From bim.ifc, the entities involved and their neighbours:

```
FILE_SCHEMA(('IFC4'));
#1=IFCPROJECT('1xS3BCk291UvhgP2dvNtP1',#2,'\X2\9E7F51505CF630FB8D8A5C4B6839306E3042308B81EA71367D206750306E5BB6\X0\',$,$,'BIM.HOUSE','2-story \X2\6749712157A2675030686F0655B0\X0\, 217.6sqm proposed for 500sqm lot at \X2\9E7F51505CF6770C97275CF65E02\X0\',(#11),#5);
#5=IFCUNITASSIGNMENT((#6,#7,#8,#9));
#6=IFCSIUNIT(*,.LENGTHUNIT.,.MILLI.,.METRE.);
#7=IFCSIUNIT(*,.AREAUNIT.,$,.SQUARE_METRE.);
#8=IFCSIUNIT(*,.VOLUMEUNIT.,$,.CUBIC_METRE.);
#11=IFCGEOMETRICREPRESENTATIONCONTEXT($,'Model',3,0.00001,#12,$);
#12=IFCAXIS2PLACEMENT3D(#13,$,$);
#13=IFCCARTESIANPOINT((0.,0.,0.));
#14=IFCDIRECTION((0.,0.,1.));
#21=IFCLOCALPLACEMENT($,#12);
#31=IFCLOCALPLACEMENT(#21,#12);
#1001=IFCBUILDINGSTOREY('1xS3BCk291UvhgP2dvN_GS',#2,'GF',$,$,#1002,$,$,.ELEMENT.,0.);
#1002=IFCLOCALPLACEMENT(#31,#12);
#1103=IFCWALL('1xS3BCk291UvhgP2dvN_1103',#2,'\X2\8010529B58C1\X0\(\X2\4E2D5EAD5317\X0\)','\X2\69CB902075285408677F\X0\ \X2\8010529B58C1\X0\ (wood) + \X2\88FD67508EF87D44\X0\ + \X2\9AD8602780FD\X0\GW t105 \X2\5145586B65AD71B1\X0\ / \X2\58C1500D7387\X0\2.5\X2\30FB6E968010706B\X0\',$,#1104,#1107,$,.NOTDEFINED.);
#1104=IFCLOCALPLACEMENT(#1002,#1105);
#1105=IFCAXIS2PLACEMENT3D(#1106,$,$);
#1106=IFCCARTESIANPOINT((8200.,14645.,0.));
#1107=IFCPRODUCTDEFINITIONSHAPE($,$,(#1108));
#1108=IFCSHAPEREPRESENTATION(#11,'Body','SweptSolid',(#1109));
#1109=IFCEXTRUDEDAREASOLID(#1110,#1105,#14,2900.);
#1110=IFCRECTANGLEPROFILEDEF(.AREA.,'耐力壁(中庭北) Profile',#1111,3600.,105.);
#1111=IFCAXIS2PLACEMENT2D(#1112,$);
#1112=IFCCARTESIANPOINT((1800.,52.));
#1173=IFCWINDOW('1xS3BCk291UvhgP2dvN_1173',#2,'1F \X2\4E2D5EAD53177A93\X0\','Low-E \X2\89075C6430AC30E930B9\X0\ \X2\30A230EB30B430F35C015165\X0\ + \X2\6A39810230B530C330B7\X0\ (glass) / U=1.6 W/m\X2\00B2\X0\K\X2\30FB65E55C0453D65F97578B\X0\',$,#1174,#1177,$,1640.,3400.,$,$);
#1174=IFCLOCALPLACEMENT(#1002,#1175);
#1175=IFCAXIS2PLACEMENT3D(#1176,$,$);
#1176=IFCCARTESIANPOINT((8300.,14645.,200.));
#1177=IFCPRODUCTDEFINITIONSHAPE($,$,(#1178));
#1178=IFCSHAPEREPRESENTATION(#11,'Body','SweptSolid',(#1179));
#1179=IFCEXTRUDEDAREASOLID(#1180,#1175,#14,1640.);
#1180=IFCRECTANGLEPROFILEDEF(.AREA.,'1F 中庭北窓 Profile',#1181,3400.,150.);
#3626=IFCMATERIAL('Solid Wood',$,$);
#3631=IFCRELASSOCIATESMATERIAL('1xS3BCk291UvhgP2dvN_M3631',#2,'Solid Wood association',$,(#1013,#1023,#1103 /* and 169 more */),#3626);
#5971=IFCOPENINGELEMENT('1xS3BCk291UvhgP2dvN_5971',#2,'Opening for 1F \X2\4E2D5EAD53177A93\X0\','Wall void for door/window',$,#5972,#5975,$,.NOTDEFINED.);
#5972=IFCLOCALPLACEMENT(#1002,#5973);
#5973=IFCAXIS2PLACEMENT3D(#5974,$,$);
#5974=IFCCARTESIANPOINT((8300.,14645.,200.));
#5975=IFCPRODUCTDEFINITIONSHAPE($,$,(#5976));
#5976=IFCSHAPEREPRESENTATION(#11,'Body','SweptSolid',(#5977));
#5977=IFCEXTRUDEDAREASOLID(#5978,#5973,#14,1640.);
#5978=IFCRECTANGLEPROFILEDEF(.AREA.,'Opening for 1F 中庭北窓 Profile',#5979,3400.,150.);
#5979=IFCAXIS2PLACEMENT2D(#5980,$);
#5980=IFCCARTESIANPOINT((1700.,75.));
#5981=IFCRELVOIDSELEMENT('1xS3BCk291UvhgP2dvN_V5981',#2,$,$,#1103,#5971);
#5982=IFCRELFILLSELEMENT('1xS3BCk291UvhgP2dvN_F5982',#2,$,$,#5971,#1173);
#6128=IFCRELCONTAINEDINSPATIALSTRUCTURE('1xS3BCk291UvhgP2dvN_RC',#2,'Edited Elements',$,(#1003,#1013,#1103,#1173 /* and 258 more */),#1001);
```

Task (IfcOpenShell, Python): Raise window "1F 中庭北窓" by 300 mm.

```python
import numpy as np
import ifcopenshell
import ifcopenshell.api.geometry
import ifcopenshell.util.placement
import ifcopenshell.util.unit

model = ifcopenshell.open("bim.ifc")
unit_scale = ifcopenshell.util.unit.calculate_unit_scale(model)

window = model.by_guid("1xS3BCk291UvhgP2dvN_1173")
opening = window.FillsVoids[0].RelatingOpeningElement
dz = 300.0

shift = np.array([0.0, 0.0, dz])
# The window is not placed relative to its opening, so move both.
for product in (opening, window):
    matrix = ifcopenshell.util.placement.get_local_placement(product.ObjectPlacement)
    matrix[:3, 3] += shift
    ifcopenshell.api.geometry.edit_object_placement(model, product=product, matrix=matrix, is_si=False)

print(f"moved by {dz * unit_scale:+.3f} m")

model.write("bim-out.ifc")
```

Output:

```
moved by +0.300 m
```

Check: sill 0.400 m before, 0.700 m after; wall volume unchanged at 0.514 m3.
